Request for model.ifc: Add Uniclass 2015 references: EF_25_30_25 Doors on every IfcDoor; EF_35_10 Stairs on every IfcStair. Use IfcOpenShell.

First a look at what the model holds.

```python
import ifcopenshell

model = ifcopenshell.open("model.ifc")
print(model.schema)
print("classifications:", [c.Name for c in model.by_type("IfcClassification")])
for ifc_class in ("IfcDoor", "IfcRoof", "IfcStair", "IfcWall", "IfcWindow"):
    print(ifc_class, len(model.by_type(ifc_class)))
```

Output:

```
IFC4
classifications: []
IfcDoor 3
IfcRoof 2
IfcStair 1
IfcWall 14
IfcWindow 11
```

```python
import ifcopenshell
import ifcopenshell.api.classification

model = ifcopenshell.open("model.ifc")

system = ifcopenshell.api.classification.add_classification(model, classification="Uniclass 2015")

codes = {
    "IfcDoor": ("EF_25_30_25", "Doors"),
    "IfcStair": ("EF_35_10", "Stairs"),
}
for ifc_class, (code, name) in codes.items():
    products = model.by_type(ifc_class)
    ifcopenshell.api.classification.add_reference(
        model, products=products, classification=system, identification=code, name=name
    )
    print(code, len(products))

model.write("model_updated.ifc")
```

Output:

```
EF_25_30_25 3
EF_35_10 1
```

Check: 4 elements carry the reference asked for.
